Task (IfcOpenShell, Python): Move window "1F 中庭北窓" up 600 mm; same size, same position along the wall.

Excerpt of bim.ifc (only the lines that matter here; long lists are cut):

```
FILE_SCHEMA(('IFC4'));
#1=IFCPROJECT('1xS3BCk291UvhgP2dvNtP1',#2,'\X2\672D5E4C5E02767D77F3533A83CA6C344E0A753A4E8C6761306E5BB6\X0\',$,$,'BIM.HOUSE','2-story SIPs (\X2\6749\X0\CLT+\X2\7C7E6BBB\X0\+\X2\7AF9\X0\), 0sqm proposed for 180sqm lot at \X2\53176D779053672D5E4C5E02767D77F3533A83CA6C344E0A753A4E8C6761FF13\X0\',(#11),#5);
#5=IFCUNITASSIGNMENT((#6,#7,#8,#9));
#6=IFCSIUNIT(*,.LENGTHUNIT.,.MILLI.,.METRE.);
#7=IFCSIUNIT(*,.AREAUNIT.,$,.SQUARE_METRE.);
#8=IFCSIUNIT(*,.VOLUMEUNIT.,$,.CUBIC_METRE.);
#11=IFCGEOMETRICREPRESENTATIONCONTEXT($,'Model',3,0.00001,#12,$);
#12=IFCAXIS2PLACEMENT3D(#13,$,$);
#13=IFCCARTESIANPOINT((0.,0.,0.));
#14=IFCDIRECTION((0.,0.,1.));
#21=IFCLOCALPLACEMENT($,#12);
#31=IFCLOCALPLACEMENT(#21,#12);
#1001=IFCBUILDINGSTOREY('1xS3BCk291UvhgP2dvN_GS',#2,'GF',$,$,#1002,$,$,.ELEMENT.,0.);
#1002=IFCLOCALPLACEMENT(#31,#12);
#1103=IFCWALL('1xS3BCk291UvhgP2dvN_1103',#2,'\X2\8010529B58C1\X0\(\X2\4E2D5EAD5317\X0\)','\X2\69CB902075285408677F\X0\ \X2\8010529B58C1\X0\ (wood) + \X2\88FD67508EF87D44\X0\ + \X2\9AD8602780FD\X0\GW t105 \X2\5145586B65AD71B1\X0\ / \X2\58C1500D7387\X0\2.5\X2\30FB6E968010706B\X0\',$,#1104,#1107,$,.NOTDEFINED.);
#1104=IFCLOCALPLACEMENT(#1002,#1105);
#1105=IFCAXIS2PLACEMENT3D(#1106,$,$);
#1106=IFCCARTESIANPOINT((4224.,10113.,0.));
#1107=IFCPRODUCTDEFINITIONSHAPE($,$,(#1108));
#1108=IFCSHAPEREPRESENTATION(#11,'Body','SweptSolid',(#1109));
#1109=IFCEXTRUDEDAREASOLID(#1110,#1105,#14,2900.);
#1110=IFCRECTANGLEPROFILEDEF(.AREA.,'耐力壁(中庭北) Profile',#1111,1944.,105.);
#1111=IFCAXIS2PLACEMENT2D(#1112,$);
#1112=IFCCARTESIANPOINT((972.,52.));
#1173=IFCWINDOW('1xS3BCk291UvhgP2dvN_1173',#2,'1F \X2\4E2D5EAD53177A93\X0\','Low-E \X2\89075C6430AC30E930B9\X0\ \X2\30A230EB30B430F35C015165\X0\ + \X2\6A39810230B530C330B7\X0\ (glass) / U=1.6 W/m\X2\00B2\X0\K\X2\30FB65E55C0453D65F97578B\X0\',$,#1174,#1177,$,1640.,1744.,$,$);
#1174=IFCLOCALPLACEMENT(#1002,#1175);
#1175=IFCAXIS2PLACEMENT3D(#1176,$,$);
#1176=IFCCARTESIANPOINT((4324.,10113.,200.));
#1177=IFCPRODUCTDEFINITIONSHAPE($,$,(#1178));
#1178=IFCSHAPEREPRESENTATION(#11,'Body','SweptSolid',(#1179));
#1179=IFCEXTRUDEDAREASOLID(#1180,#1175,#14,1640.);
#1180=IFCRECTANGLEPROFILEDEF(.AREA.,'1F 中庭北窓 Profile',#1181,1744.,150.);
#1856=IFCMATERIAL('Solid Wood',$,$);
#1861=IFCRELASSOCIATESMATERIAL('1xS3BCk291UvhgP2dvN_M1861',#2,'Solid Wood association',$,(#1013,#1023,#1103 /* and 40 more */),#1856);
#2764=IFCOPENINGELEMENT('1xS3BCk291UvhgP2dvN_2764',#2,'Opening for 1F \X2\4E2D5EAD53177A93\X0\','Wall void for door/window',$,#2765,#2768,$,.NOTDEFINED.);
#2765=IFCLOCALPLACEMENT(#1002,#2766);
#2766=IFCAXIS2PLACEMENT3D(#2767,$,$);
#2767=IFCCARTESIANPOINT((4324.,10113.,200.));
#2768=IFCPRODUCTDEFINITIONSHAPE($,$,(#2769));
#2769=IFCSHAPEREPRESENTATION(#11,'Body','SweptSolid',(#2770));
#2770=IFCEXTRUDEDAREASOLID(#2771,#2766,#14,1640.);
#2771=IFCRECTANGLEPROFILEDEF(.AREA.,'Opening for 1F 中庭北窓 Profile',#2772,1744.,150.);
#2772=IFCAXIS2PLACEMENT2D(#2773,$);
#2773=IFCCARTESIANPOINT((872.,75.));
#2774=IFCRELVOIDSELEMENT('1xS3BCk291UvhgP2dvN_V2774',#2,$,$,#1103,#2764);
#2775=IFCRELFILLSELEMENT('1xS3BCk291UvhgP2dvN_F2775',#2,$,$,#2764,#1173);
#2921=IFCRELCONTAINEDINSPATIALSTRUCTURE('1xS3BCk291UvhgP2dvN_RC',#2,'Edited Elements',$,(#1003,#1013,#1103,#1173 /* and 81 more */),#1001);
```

```python
import numpy as np
import ifcopenshell
import ifcopenshell.api.geometry
import ifcopenshell.util.placement
import ifcopenshell.util.unit

model = ifcopenshell.open("bim.ifc")
unit_scale = ifcopenshell.util.unit.calculate_unit_scale(model)

window = model.by_guid("1xS3BCk291UvhgP2dvN_1173")
opening = window.FillsVoids[0].RelatingOpeningElement
dz = 0.6 / unit_scale

shift = np.array([0.0, 0.0, dz])
# The window is not placed relative to its opening, so move both.
for product in (opening, window):
    matrix = ifcopenshell.util.placement.get_local_placement(product.ObjectPlacement)
    matrix[:3, 3] += shift
    ifcopenshell.api.geometry.edit_object_placement(model, product=product, matrix=matrix, is_si=False)

print(f"moved by {dz * unit_scale:+.3f} m")

model.write("bim_edited.ifc")
```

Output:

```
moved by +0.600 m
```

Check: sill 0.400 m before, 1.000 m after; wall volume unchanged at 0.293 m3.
